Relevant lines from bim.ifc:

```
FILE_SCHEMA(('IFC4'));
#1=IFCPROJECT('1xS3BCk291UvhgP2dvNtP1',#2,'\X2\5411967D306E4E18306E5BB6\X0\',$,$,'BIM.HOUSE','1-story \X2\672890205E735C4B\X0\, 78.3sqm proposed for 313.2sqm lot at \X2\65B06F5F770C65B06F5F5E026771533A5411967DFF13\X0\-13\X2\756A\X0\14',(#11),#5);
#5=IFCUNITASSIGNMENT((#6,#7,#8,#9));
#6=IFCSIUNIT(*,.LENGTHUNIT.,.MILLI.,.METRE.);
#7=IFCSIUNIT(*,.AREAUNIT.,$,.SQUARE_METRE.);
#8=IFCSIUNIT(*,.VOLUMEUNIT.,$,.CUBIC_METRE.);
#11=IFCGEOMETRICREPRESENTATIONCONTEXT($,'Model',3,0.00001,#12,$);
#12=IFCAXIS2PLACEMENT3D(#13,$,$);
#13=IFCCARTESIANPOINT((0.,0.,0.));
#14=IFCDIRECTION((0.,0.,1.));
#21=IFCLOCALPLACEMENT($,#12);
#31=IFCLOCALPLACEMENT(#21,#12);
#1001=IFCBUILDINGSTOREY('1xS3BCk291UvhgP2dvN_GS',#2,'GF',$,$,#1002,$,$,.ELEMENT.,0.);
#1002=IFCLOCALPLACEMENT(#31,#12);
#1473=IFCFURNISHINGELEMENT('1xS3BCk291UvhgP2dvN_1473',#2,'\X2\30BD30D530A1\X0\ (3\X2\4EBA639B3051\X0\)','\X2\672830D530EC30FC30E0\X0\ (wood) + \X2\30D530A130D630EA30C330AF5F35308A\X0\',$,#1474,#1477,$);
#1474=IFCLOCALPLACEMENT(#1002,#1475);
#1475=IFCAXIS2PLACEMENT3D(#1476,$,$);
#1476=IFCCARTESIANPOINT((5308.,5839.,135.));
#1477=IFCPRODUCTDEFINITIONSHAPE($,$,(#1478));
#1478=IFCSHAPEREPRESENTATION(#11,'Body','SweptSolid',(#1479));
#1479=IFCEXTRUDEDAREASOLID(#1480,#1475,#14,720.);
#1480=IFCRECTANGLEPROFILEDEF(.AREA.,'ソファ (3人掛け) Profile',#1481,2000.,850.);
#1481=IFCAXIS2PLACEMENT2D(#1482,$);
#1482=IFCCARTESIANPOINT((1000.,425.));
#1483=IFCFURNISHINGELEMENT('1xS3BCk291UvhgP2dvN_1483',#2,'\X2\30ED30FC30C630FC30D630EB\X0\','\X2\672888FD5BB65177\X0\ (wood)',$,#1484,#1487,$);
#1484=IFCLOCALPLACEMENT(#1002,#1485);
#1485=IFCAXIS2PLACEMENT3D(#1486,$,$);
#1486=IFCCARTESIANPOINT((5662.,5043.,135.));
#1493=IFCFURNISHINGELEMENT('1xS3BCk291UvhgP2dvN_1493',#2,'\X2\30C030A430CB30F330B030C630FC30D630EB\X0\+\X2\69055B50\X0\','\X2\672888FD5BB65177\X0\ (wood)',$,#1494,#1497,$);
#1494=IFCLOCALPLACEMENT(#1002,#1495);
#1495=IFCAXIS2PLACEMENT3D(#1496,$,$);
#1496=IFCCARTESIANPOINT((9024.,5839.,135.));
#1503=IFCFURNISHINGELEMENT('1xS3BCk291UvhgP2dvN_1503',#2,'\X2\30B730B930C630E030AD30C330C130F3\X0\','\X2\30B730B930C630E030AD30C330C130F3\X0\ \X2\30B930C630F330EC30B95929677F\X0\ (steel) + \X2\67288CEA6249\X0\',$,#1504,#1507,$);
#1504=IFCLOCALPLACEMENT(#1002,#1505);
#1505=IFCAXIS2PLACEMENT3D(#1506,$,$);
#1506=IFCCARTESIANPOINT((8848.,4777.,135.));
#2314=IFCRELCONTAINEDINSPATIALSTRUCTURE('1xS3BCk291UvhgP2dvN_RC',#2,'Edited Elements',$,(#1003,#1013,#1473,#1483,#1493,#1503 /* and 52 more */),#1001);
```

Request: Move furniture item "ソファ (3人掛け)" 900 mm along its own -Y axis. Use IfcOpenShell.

```python
import ifcopenshell
import ifcopenshell.api.geometry
import ifcopenshell.util.placement
import ifcopenshell.util.unit

model = ifcopenshell.open("bim.ifc")
unit_scale = ifcopenshell.util.unit.calculate_unit_scale(model)

item = model.by_id(1473)
matrix = ifcopenshell.util.placement.get_local_placement(item.ObjectPlacement)
matrix[:3, 3] -= matrix[:3, 1] * 0.9 / unit_scale
ifcopenshell.api.geometry.edit_object_placement(model, product=item, matrix=matrix, is_si=False)

print(ifcopenshell.util.placement.get_local_placement(item.ObjectPlacement).round(3) + 0.0)

model.write("bim_v2.ifc")
```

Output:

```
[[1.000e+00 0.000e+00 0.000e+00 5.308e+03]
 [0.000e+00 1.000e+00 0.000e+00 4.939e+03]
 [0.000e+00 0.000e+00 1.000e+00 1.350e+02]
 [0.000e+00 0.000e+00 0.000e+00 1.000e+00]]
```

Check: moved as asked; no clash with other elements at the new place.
